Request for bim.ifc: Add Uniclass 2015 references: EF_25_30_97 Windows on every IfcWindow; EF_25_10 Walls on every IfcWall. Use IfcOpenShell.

First a look at what the model holds.

```python
import ifcopenshell

model = ifcopenshell.open("bim.ifc")
print(model.schema)
print("classifications:", [c.Name for c in model.by_type("IfcClassification")])
for ifc_class in ("IfcDoor", "IfcRoof", "IfcStair", "IfcWall", "IfcWindow"):
    print(ifc_class, len(model.by_type(ifc_class)))
```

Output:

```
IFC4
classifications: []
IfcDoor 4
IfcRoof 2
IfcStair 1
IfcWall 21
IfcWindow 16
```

```python
import ifcopenshell
import ifcopenshell.api.classification

model = ifcopenshell.open("bim.ifc")

system = ifcopenshell.api.classification.add_classification(model, classification="Uniclass 2015")

codes = {
    "IfcWindow": ("EF_25_30_97", "Windows"),
    "IfcWall": ("EF_25_10", "Walls"),
}
for ifc_class, (code, name) in codes.items():
    products = model.by_type(ifc_class)
    ifcopenshell.api.classification.add_reference(
        model, products=products, classification=system, identification=code, name=name
    )
    print(code, len(products))

model.write("bim_updated.ifc")
```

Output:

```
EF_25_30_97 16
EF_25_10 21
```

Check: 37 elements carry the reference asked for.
